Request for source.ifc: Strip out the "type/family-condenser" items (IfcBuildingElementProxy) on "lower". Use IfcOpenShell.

First a look at what the model holds.

```python
import ifcopenshell
import ifcopenshell.util.element

model = ifcopenshell.open("source.ifc")
print(model.schema)
storey = next(s for s in model.by_type("IfcBuildingStorey") if s.Name == "lower")
proxies = [e for e in ifcopenshell.util.element.get_decomposition(storey) if e.is_a("IfcBuildingElementProxy")]
seen = {}
for e in proxies:
    element_type = ifcopenshell.util.element.get_type(e)
    name = element_type.Name if element_type not in (None, e) else None
    seen[name] = seen.get(name, 0) + 1
for name, count in sorted(seen.items(), key=str):
    print(count, "x", name)
```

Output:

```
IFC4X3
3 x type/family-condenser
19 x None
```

```python
import ifcopenshell
import ifcopenshell.api.root
import ifcopenshell.util.element

model = ifcopenshell.open("source.ifc")

storey = next(s for s in model.by_type("IfcBuildingStorey") if s.Name == "lower")
proxies = [e for e in ifcopenshell.util.element.get_decomposition(storey) if e.is_a("IfcBuildingElementProxy")]
targets = [e for e in proxies if (t := ifcopenshell.util.element.get_type(e)) not in (None, e) and t.Name == "type/family-condenser"]

for e in targets:
    ifcopenshell.api.root.remove_product(model, product=e)
print(len(targets), "removed")

model.write("source_rev.ifc")
```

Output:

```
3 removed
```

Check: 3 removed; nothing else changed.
